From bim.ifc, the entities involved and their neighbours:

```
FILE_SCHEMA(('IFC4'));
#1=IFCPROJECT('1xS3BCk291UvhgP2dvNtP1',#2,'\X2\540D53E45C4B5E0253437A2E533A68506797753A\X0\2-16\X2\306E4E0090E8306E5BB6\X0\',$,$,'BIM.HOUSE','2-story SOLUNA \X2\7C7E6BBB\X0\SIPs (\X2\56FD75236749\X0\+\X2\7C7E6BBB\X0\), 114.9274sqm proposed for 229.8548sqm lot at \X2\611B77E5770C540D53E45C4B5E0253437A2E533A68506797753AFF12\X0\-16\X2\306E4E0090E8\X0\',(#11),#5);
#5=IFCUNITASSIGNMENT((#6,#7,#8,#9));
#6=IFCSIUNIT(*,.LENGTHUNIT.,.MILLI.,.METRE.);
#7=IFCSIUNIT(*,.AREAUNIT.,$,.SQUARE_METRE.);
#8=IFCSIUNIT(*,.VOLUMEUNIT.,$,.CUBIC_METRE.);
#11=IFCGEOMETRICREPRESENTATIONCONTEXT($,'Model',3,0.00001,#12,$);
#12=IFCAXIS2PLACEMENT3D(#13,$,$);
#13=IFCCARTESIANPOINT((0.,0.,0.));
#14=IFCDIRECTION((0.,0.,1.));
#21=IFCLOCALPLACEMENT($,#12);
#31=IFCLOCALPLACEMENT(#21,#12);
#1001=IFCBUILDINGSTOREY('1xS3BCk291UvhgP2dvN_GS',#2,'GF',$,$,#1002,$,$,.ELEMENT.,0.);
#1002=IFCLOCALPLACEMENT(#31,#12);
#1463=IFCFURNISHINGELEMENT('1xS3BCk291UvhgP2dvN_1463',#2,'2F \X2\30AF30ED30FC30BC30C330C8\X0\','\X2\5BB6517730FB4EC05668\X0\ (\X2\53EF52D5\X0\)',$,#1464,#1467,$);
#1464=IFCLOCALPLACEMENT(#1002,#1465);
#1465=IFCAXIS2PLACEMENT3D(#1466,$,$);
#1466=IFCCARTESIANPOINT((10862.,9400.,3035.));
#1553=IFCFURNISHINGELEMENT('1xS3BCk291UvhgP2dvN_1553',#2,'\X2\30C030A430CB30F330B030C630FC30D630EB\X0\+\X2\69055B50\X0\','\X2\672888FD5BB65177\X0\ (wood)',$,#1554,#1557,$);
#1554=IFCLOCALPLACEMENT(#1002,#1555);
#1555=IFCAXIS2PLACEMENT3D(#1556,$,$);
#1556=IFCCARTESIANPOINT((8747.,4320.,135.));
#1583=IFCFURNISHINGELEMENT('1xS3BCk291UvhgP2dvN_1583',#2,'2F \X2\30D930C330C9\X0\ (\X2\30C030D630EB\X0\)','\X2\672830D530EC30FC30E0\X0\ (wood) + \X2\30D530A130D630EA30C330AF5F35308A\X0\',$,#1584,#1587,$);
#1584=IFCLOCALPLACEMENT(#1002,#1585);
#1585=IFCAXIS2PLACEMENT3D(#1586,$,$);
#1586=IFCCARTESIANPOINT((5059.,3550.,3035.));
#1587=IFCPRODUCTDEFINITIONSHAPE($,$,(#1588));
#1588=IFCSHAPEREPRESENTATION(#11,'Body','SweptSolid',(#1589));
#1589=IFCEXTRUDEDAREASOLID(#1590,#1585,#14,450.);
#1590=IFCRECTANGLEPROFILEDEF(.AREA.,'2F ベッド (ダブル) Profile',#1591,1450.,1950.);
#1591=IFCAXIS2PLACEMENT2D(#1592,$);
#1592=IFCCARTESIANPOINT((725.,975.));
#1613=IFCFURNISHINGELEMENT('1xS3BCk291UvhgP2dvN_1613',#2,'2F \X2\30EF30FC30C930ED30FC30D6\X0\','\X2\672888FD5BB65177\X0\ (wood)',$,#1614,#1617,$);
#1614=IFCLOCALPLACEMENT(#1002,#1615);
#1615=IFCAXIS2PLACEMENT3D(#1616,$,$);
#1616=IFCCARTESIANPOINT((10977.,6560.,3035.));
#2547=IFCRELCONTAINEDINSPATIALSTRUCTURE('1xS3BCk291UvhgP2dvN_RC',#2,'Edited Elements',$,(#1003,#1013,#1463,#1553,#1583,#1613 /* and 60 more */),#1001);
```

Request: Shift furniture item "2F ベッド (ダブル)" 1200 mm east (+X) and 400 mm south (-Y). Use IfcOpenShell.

```python
import ifcopenshell
import ifcopenshell.api.geometry
import ifcopenshell.util.placement
import ifcopenshell.util.unit

model = ifcopenshell.open("bim.ifc")
unit_scale = ifcopenshell.util.unit.calculate_unit_scale(model)

item = model.by_guid("1xS3BCk291UvhgP2dvN_1583")
matrix = ifcopenshell.util.placement.get_local_placement(item.ObjectPlacement)
matrix[0, 3] += 1.2 / unit_scale
matrix[1, 3] -= 0.4 / unit_scale
ifcopenshell.api.geometry.edit_object_placement(model, product=item, matrix=matrix, is_si=False)

print(ifcopenshell.util.placement.get_local_placement(item.ObjectPlacement).round(3) + 0.0)

model.write("bim_updated.ifc")
```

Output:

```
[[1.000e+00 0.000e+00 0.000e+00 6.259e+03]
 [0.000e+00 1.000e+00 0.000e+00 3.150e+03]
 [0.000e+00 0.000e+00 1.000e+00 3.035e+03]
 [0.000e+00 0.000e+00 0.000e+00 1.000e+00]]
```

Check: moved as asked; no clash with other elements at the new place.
